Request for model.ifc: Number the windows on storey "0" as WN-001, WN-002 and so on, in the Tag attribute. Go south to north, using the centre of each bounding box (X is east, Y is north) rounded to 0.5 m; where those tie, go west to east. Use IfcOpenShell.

First a look at what the model holds.

```python
import ifcopenshell
import ifcopenshell.util.element
import ifcopenshell.util.placement

model = ifcopenshell.open("model.ifc")
print(model.schema)
storey = next(s for s in model.by_type("IfcBuildingStorey") if s.Name == "0")
windows = [e for e in ifcopenshell.util.element.get_decomposition(storey) if e.is_a("IfcWindow")]
for e in sorted(windows, key=lambda e: e.id()):
    origin = ifcopenshell.util.placement.get_local_placement(e.ObjectPlacement)[:3, 3]
    print(e.id(), e.Tag, e.Name, origin.round(2) + 0.0, sep=" | ")
```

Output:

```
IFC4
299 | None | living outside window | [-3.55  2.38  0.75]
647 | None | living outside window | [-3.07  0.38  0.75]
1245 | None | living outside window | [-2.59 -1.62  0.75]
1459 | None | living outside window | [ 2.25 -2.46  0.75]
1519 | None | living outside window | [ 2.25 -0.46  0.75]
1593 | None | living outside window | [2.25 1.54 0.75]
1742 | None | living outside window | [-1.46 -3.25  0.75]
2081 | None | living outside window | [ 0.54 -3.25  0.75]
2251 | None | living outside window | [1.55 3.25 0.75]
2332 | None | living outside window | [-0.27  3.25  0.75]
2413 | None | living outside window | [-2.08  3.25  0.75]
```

```python
import ifcopenshell
import ifcopenshell.geom
import ifcopenshell.util.element
import ifcopenshell.util.shape

model = ifcopenshell.open("model.ifc")
settings = ifcopenshell.geom.settings()
settings.set("use-world-coords", True)


def centre(element):
    shape = ifcopenshell.geom.create_shape(settings, element)
    return ifcopenshell.util.shape.get_bbox_centroid(shape.geometry)


storey = next(s for s in model.by_type("IfcBuildingStorey") if s.Name == "0")
windows = [e for e in ifcopenshell.util.element.get_decomposition(storey) if e.is_a("IfcWindow")]

# Insertion points can sit at a corner or the storey origin, so sort by the geometry (in metres).
centres = {e: centre(e) for e in windows}
windows.sort(key=lambda e: (round(centres[e][1] / 0.5), centres[e][0]))

for i, e in enumerate(windows, start=1):
    number = f"WN-0{i:02d}"
    e.Tag = number
    print(e.id(), number)

model.write("model_rev.ifc")
```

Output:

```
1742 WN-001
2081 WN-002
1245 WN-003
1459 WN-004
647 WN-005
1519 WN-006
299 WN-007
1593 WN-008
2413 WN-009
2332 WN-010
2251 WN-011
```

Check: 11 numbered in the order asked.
